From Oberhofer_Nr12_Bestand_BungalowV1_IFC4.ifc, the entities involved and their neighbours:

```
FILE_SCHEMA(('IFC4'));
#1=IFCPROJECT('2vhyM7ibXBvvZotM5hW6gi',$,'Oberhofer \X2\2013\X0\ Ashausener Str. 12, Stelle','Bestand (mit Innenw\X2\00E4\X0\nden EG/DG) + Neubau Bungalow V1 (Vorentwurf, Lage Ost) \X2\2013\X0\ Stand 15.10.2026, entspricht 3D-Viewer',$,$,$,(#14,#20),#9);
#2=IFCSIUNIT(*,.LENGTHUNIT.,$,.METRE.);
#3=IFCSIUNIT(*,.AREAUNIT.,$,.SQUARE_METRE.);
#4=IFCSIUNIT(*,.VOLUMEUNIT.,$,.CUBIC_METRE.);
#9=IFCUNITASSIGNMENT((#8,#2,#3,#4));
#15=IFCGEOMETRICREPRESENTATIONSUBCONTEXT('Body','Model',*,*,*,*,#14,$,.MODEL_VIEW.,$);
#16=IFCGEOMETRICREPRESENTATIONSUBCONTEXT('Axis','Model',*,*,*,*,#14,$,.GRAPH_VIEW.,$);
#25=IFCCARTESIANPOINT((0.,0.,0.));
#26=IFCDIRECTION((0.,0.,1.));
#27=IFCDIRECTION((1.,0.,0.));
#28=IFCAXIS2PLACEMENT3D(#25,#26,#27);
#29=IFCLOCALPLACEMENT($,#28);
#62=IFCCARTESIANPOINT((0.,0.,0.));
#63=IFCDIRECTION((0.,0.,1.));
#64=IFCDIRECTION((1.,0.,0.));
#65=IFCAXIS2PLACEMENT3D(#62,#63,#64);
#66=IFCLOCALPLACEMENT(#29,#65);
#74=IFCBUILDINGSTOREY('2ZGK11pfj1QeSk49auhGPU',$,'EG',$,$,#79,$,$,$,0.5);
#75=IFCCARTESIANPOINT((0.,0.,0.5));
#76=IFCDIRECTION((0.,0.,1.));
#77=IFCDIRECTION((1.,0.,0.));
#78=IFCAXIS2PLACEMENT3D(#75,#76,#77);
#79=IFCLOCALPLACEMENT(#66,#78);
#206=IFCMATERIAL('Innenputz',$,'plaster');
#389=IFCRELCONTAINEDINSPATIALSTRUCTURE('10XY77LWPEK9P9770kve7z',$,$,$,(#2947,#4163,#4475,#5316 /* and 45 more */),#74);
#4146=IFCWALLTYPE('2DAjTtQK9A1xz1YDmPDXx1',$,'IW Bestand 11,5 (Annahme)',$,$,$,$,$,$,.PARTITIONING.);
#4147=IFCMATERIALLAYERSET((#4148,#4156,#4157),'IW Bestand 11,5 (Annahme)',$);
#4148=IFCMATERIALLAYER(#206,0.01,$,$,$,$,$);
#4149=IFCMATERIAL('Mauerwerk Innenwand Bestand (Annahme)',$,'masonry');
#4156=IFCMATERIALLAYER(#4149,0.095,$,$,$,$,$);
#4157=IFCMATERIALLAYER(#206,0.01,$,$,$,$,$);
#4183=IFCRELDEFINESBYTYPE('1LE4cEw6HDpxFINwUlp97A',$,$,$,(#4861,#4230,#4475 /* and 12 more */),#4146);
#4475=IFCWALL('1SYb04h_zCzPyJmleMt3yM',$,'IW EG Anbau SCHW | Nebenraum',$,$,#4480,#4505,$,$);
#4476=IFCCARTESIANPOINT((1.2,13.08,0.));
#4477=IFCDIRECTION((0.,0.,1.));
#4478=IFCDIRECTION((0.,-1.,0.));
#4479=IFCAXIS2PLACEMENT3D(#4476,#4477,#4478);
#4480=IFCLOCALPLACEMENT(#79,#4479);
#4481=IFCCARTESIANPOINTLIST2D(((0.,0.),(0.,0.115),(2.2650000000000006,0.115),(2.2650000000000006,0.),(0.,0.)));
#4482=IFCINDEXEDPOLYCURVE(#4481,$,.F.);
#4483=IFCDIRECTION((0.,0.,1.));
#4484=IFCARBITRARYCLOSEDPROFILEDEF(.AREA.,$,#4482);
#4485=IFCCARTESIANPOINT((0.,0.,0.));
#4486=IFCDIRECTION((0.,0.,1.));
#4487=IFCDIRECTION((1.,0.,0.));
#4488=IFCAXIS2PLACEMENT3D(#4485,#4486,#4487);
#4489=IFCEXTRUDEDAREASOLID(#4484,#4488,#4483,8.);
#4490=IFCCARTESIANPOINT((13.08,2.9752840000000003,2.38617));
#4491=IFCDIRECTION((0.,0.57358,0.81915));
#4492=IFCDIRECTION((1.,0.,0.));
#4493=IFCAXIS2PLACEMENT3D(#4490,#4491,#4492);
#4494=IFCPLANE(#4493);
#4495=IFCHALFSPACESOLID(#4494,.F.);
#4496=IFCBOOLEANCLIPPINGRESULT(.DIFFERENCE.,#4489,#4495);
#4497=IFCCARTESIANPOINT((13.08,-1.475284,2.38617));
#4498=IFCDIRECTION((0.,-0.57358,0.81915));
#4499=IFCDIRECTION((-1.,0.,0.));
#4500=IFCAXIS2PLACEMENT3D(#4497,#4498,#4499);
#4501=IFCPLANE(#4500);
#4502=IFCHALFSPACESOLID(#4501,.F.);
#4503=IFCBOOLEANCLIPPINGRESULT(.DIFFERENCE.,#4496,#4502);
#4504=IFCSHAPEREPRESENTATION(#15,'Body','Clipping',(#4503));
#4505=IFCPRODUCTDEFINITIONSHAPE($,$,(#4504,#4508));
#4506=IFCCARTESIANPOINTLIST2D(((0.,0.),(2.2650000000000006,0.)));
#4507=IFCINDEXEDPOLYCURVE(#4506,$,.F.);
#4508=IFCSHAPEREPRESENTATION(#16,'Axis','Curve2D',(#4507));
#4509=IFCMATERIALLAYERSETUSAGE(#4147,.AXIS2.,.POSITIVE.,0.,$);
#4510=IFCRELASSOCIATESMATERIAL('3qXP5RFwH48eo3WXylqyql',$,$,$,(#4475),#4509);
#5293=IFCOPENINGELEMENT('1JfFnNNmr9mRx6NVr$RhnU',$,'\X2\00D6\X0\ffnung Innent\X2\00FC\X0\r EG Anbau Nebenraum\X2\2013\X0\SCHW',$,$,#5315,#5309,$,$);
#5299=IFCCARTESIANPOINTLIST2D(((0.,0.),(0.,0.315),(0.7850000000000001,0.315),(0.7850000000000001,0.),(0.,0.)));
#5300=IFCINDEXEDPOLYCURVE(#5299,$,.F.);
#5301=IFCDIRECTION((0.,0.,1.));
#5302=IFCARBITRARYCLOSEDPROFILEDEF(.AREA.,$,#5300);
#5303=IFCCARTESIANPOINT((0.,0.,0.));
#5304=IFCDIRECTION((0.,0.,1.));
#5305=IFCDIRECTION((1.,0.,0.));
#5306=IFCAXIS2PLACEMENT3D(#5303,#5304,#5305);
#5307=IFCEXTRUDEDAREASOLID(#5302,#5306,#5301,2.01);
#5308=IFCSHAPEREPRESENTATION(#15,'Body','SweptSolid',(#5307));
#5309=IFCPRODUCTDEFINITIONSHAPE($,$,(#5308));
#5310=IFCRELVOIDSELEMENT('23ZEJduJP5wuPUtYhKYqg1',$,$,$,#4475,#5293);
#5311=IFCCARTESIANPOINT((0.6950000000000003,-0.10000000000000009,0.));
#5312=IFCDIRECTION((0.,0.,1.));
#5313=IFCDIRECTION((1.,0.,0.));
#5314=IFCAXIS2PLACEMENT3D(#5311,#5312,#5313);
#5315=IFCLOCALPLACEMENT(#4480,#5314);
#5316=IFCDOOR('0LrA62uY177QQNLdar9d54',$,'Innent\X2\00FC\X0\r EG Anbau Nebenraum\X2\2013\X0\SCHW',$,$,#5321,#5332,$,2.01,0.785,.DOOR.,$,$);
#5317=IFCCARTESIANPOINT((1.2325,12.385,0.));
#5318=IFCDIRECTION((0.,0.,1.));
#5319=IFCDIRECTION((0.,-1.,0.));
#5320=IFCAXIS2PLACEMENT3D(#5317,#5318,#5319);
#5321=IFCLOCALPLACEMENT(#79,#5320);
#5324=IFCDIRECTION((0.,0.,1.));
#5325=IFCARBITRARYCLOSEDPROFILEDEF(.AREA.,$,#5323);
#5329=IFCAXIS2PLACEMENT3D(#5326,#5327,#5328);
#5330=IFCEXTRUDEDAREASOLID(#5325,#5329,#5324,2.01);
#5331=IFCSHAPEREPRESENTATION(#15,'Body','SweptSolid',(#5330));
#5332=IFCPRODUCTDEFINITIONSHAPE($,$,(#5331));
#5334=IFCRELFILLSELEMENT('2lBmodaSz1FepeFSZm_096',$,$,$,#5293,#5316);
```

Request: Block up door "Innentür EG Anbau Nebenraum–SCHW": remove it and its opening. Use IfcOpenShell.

```python
import ifcopenshell
import ifcopenshell.api.feature
import ifcopenshell.api.root
import ifcopenshell.geom
import ifcopenshell.util.shape

model = ifcopenshell.open("Oberhofer_Nr12_Bestand_BungalowV1_IFC4.ifc")
settings = ifcopenshell.geom.settings()


def volume(element):
    """Net volume in cubic metres, openings subtracted."""
    shape = ifcopenshell.geom.create_shape(settings, element)
    return ifcopenshell.util.shape.get_volume(shape.geometry)


door = model.by_guid("0LrA62uY177QQNLdar9d54")
opening = door.FillsVoids[0].RelatingOpeningElement
wall = opening.VoidsElements[0].RelatingBuildingElement
before = volume(wall)

ifcopenshell.api.root.remove_product(model, product=door)
ifcopenshell.api.feature.remove_feature(model, feature=opening)

after = volume(wall)

print(f"wall volume {before:.3f} -> {after:.3f} m3")

model.write("Oberhofer_Nr12_Bestand_BungalowV1_IFC4_edited.ifc")
```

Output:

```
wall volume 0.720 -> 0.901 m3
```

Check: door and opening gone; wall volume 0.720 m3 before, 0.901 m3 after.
